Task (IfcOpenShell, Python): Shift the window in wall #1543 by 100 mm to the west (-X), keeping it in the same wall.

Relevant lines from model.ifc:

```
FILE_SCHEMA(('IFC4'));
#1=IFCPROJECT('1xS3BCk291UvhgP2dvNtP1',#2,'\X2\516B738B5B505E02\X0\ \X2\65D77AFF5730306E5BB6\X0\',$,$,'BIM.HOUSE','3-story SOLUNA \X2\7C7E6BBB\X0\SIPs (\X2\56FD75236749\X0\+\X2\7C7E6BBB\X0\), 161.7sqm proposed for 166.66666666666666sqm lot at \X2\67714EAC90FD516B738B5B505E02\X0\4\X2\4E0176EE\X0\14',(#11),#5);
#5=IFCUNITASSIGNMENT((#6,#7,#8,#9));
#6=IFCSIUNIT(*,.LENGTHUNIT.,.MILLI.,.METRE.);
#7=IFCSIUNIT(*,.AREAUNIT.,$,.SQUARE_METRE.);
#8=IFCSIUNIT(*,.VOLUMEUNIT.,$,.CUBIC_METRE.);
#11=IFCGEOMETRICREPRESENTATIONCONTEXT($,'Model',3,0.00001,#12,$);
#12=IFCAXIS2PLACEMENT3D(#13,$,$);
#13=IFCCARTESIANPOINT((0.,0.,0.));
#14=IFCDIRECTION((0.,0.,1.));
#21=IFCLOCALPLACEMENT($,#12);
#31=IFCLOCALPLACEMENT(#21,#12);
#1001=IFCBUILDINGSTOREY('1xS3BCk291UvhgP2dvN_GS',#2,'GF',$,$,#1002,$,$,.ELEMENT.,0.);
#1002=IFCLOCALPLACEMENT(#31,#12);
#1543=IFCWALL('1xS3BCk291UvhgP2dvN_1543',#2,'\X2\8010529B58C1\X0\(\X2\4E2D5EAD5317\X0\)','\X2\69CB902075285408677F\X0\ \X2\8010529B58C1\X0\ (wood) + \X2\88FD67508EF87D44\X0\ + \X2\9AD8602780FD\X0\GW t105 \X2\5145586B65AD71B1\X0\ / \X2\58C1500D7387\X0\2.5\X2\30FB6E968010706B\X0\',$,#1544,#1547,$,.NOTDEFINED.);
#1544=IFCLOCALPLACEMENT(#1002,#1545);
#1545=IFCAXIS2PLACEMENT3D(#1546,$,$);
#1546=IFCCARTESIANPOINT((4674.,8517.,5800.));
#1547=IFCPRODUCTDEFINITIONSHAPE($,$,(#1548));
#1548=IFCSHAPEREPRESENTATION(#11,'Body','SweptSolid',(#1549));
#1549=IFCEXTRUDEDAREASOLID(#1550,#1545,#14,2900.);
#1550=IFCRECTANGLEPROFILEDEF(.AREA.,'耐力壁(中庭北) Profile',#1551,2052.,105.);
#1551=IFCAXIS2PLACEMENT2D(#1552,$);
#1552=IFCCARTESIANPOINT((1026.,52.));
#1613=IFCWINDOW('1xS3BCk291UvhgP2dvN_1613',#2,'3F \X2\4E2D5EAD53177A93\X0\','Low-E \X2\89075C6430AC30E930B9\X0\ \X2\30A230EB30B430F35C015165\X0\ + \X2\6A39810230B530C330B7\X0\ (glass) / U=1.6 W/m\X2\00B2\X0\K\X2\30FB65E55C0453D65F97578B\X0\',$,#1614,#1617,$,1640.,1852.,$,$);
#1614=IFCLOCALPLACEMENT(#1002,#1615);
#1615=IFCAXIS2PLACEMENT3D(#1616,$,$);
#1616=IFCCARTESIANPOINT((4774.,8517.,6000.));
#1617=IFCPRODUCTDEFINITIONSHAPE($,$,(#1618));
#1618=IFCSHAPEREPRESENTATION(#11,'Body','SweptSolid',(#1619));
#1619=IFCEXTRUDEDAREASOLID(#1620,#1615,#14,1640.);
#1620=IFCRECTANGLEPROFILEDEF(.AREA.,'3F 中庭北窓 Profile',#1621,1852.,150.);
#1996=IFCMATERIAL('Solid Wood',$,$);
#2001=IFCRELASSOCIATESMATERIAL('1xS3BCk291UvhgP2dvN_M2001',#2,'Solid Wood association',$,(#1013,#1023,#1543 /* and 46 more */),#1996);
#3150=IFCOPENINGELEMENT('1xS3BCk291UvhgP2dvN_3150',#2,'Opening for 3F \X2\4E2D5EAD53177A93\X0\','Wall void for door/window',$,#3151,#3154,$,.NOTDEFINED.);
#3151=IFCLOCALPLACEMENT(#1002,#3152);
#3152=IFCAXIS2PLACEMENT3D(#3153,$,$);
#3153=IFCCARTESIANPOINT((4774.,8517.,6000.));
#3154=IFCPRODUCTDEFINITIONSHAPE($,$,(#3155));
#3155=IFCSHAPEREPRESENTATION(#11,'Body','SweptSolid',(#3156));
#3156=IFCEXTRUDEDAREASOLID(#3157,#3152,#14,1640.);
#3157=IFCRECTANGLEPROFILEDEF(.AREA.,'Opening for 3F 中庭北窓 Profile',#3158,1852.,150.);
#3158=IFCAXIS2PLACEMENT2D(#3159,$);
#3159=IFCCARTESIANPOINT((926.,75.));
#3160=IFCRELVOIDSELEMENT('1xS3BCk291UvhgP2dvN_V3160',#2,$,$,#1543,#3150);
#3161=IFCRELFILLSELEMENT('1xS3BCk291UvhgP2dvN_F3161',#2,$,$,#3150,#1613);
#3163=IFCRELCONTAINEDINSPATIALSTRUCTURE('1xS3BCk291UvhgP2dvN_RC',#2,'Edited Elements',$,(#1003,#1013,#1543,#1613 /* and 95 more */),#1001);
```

```python
import ifcopenshell
import ifcopenshell.api.geometry
import ifcopenshell.util.placement
import ifcopenshell.util.unit

model = ifcopenshell.open("model.ifc")
unit_scale = ifcopenshell.util.unit.calculate_unit_scale(model)

window = model.by_guid("1xS3BCk291UvhgP2dvN_1613")
opening = window.FillsVoids[0].RelatingOpeningElement
wall = opening.VoidsElements[0].RelatingBuildingElement

wall_matrix = ifcopenshell.util.placement.get_local_placement(wall.ObjectPlacement)
shift = wall_matrix[:3, 0] * -0.1 / unit_scale
before = ifcopenshell.util.placement.get_local_placement(window.ObjectPlacement)[:3, 3].copy()

# The window is not placed relative to its opening, so move both.
for product in (opening, window):
    matrix = ifcopenshell.util.placement.get_local_placement(product.ObjectPlacement)
    matrix[:3, 3] += shift
    ifcopenshell.api.geometry.edit_object_placement(model, product=product, matrix=matrix, is_si=False)

after = ifcopenshell.util.placement.get_local_placement(window.ObjectPlacement)[:3, 3]
print("window moved by", (after - before).round(3) + 0.0)

model.write("model_rev.ifc")
```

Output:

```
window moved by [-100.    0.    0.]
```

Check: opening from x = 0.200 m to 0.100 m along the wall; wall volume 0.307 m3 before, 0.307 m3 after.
